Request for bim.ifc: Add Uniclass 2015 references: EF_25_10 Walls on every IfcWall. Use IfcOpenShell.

First a look at what the model holds.

```python
import ifcopenshell

model = ifcopenshell.open("bim.ifc")
print(model.schema)
print("classifications:", [c.Name for c in model.by_type("IfcClassification")])
for ifc_class in ("IfcDoor", "IfcRoof", "IfcStair", "IfcWall", "IfcWindow"):
    print(ifc_class, len(model.by_type(ifc_class)))
```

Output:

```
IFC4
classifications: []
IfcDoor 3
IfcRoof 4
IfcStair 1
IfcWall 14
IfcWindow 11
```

```python
import ifcopenshell
import ifcopenshell.api.classification

model = ifcopenshell.open("bim.ifc")

system = ifcopenshell.api.classification.add_classification(model, classification="Uniclass 2015")

codes = {
    "IfcWall": ("EF_25_10", "Walls"),
}
for ifc_class, (code, name) in codes.items():
    products = model.by_type(ifc_class)
    ifcopenshell.api.classification.add_reference(
        model, products=products, classification=system, identification=code, name=name
    )
    print(code, len(products))

model.write("bim_v2.ifc")
```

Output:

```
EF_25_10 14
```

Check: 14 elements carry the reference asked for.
